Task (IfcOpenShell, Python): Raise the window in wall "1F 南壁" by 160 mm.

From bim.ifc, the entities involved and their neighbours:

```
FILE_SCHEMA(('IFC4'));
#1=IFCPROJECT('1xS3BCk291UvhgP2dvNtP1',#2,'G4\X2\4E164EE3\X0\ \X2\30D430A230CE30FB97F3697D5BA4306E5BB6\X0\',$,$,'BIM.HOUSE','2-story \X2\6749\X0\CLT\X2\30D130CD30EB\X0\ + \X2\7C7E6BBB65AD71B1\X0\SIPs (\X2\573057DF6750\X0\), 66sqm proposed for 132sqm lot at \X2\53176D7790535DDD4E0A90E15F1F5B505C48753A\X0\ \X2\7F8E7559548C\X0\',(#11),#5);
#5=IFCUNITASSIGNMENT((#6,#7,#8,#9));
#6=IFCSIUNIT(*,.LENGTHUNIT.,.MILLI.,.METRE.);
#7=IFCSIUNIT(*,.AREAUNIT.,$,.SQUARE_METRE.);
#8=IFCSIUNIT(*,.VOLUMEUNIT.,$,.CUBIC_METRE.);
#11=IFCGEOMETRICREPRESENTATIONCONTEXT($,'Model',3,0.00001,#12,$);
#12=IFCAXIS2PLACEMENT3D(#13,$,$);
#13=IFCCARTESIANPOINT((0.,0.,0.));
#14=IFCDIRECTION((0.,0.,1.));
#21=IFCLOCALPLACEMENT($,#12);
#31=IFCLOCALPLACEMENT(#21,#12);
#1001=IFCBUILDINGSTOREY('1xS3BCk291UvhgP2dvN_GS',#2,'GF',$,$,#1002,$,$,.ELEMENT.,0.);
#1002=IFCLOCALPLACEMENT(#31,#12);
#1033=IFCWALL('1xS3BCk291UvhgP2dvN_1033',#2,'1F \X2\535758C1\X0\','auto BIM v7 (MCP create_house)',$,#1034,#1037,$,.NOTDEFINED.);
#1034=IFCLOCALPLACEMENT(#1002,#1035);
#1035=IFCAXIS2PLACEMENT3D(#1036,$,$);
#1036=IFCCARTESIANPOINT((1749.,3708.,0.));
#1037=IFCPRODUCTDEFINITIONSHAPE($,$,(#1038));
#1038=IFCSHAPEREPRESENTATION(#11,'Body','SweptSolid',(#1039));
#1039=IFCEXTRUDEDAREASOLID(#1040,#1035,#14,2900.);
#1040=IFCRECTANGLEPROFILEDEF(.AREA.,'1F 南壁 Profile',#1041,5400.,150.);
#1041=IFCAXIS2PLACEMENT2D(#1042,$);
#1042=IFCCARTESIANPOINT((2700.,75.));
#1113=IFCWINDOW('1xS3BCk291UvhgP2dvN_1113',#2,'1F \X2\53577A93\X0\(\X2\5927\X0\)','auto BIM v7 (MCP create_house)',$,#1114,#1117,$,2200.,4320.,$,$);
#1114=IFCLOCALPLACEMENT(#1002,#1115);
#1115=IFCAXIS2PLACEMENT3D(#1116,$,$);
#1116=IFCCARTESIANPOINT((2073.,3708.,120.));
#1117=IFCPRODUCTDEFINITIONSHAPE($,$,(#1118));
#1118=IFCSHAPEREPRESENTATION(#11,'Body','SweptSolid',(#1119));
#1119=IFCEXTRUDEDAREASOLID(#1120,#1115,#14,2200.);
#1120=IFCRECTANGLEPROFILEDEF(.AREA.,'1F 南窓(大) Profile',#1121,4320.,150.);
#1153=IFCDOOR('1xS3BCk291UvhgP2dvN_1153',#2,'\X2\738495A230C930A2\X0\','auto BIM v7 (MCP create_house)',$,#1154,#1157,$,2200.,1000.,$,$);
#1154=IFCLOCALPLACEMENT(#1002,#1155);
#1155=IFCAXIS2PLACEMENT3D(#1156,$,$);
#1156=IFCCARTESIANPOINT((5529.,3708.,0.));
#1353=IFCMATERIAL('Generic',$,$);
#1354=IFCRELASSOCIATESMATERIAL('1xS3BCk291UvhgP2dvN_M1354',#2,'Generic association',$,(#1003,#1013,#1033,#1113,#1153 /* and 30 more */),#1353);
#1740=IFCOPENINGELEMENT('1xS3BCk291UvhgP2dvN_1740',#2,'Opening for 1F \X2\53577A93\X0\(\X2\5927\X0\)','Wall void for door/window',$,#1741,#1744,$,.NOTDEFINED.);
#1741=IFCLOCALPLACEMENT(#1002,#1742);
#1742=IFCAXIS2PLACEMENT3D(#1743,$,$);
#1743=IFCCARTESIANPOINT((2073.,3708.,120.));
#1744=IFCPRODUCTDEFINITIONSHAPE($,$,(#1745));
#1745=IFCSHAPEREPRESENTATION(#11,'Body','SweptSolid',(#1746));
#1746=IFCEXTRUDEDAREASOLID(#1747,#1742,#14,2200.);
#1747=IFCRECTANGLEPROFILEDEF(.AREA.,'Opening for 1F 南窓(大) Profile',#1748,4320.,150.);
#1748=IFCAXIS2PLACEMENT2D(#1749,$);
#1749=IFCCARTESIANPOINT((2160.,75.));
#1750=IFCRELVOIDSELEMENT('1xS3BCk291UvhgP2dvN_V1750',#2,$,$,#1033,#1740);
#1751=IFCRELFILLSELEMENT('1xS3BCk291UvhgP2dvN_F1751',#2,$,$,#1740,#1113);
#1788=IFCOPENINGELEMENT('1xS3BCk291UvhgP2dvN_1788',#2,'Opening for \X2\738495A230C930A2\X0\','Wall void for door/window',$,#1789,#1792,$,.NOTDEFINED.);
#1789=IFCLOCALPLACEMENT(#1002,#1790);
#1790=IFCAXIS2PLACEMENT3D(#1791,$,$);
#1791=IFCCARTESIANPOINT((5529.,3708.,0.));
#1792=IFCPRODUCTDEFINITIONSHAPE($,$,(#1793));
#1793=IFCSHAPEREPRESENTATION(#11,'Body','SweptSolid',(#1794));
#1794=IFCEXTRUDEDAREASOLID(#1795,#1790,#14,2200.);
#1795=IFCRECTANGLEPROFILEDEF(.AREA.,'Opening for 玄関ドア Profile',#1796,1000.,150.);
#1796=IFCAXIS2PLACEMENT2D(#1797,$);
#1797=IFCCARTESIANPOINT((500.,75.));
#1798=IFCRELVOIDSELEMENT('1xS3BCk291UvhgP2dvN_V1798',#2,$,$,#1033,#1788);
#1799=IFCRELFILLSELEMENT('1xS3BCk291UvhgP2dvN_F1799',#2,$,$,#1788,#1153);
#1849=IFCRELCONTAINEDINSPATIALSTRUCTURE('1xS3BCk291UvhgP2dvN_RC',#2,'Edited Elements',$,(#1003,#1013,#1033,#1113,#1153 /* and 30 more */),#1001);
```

```python
import numpy as np
import ifcopenshell
import ifcopenshell.api.geometry
import ifcopenshell.util.placement
import ifcopenshell.util.unit

model = ifcopenshell.open("bim.ifc")
unit_scale = ifcopenshell.util.unit.calculate_unit_scale(model)

window = model.by_id(1113)
opening = window.FillsVoids[0].RelatingOpeningElement
dz = 0.16 / unit_scale

shift = np.array([0.0, 0.0, dz])
# The window is not placed relative to its opening, so move both.
for product in (opening, window):
    matrix = ifcopenshell.util.placement.get_local_placement(product.ObjectPlacement)
    matrix[:3, 3] += shift
    ifcopenshell.api.geometry.edit_object_placement(model, product=product, matrix=matrix, is_si=False)

print(f"moved by {dz * unit_scale:+.3f} m")

model.write("bim_v2.ifc")
```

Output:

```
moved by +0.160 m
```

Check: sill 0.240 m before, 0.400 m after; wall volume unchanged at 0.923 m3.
